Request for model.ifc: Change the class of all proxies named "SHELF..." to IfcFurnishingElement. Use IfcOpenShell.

First a look at what the model holds.

```python
import re

import ifcopenshell

model = ifcopenshell.open("model.ifc")
print(model.schema)
seen = {}
for e in model.by_type("IfcBuildingElementProxy"):
    name = re.sub(r":\d+(:\d+)?$", "", e.Name or "")  # drop the element id that some exporters append
    seen[name] = seen.get(name, 0) + 1
for name, count in sorted(seen.items()):
    print(count, "x", name)
```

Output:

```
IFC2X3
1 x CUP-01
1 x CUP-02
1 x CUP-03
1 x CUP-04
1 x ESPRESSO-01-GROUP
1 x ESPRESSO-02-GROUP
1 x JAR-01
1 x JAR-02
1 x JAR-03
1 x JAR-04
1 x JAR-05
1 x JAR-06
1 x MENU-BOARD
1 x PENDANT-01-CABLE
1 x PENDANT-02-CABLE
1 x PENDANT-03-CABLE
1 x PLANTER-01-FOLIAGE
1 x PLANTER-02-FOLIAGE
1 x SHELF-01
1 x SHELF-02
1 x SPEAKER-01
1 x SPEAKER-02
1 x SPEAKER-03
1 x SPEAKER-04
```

```python
import ifcopenshell
import ifcopenshell.api.root

model = ifcopenshell.open("model.ifc")

proxies = [e.id() for e in model.by_type("IfcBuildingElementProxy") if (e.Name or "").startswith("SHELF")]
for step_id in proxies:
    proxy = model.by_id(step_id)
    ifcopenshell.api.root.reassign_class(model, product=proxy, ifc_class="IfcFurnishingElement")

print(sum(model.by_id(i).is_a("IfcFurnishingElement") for i in proxies), "reclassified")

model.write("model_rev.ifc")
```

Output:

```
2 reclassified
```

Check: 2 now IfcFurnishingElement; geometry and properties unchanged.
